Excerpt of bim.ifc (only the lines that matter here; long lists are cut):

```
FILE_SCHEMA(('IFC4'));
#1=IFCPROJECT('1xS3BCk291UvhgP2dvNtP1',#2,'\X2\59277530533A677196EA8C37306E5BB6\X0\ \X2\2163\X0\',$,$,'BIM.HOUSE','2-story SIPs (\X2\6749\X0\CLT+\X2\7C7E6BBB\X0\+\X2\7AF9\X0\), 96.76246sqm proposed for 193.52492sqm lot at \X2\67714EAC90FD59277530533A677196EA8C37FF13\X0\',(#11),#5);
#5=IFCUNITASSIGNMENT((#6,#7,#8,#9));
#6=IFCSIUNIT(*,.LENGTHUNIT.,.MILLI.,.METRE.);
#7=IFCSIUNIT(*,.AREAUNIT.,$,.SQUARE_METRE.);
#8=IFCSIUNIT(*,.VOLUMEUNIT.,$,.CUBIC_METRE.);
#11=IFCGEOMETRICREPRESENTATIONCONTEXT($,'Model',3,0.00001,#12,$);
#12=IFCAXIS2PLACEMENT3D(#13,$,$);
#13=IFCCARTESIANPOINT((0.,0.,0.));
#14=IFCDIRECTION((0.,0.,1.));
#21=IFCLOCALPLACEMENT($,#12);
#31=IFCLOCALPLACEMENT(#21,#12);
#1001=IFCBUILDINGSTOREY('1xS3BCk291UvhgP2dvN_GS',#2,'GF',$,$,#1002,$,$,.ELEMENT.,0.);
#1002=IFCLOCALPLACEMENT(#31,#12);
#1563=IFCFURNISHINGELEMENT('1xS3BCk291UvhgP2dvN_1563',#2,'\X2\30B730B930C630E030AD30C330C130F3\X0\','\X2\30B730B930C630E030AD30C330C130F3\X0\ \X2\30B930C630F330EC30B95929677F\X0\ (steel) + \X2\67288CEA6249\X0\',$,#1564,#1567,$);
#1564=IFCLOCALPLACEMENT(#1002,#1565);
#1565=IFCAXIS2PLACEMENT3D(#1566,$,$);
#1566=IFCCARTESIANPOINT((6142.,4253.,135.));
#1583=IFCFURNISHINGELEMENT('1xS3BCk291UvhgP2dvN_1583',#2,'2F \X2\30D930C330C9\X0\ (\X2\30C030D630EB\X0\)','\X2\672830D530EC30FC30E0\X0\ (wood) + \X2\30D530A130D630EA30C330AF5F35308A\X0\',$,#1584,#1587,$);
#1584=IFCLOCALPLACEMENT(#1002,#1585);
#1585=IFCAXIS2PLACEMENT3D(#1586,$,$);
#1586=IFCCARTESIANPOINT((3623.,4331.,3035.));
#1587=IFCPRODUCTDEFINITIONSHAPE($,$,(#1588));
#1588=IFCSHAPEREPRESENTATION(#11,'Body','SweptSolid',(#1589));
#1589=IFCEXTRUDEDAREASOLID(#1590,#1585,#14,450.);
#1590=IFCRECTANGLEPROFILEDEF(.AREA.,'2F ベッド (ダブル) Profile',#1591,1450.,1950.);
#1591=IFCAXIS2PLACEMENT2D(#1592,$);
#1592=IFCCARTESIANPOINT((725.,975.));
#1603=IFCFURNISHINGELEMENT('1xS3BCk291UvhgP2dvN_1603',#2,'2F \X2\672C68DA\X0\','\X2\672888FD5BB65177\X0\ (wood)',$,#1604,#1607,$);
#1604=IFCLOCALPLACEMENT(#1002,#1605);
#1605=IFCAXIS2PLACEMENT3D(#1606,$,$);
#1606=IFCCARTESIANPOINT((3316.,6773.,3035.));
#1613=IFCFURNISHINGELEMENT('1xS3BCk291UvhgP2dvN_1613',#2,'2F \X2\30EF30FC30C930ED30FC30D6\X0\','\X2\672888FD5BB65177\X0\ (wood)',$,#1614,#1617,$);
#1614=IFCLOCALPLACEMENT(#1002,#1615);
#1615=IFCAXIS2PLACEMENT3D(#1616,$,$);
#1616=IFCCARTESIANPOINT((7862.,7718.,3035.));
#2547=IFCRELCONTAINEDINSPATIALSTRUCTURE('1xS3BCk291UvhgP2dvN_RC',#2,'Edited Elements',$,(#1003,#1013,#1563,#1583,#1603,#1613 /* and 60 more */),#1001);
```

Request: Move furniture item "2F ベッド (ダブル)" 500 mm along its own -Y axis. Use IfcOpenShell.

```python
import ifcopenshell
import ifcopenshell.api.geometry
import ifcopenshell.util.placement
import ifcopenshell.util.unit

model = ifcopenshell.open("bim.ifc")
unit_scale = ifcopenshell.util.unit.calculate_unit_scale(model)

item = model.by_guid("1xS3BCk291UvhgP2dvN_1583")
matrix = ifcopenshell.util.placement.get_local_placement(item.ObjectPlacement)
matrix[:3, 3] -= matrix[:3, 1] * 0.5 / unit_scale
ifcopenshell.api.geometry.edit_object_placement(model, product=item, matrix=matrix, is_si=False)

print(ifcopenshell.util.placement.get_local_placement(item.ObjectPlacement).round(3) + 0.0)

model.write("bim_v2.ifc")
```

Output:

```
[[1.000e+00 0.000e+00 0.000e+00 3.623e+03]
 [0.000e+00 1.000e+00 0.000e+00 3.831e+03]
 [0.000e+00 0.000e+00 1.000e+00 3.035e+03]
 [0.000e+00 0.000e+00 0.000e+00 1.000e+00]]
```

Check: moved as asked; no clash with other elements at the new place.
